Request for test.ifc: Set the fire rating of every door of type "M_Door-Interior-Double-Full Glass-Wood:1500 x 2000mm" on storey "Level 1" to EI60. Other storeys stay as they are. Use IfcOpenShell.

First a look at what the model holds.

```python
import ifcopenshell
import ifcopenshell.util.element

model = ifcopenshell.open("test.ifc")
print(model.schema)
storey = next(s for s in model.by_type("IfcBuildingStorey") if s.Name == "Level 1")
doors = [e for e in ifcopenshell.util.element.get_decomposition(storey) if e.is_a("IfcDoor")]
seen = {}
for e in doors:
    element_type = ifcopenshell.util.element.get_type(e)
    key = (element_type.Name if element_type != e and element_type else None, ifcopenshell.util.element.get_pset(e, "Pset_DoorCommon", "FireRating"))
    seen[key] = seen.get(key, 0) + 1
for (name, value), count in sorted(seen.items(), key=str):
    print(count, "x", name, "|", value)
```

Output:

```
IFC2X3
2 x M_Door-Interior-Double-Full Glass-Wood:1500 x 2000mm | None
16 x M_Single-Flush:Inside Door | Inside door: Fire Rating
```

```python
import ifcopenshell
import ifcopenshell.api.pset
import ifcopenshell.util.element

model = ifcopenshell.open("test.ifc")

storey = next(s for s in model.by_type("IfcBuildingStorey") if s.Name == "Level 1")
doors = [e for e in ifcopenshell.util.element.get_decomposition(storey) if e.is_a("IfcDoor")]

count = 0
for e in doors:
    element_type = ifcopenshell.util.element.get_type(e)
    if element_type in (None, e) or element_type.Name != "M_Door-Interior-Double-Full Glass-Wood:1500 x 2000mm":
        continue
    # add_pset returns the element's existing set when there is one.
    pset = ifcopenshell.api.pset.add_pset(model, product=e, name="Pset_DoorCommon")
    ifcopenshell.api.pset.edit_pset(model, pset=pset, properties={"FireRating": "EI60"})
    count += 1

print(count, "doors updated")

model.write("test_v2.ifc")
```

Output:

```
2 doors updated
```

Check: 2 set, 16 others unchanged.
